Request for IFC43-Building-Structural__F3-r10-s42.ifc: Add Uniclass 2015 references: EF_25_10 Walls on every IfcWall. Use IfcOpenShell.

First a look at what the model holds.

```python
import ifcopenshell

model = ifcopenshell.open("IFC43-Building-Structural__F3-r10-s42.ifc")
print(model.schema)
print("classifications:", [c.Name for c in model.by_type("IfcClassification")])
for ifc_class in ("IfcDoor", "IfcRoof", "IfcStair", "IfcWall", "IfcWindow"):
    print(ifc_class, len(model.by_type(ifc_class)))
```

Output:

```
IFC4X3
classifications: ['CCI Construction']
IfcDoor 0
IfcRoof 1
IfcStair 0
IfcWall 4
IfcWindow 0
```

```python
import ifcopenshell
import ifcopenshell.api.classification

model = ifcopenshell.open("IFC43-Building-Structural__F3-r10-s42.ifc")

system = ifcopenshell.api.classification.add_classification(model, classification="Uniclass 2015")

codes = {
    "IfcWall": ("EF_25_10", "Walls"),
}
for ifc_class, (code, name) in codes.items():
    products = model.by_type(ifc_class)
    ifcopenshell.api.classification.add_reference(
        model, products=products, classification=system, identification=code, name=name
    )
    print(code, len(products))

model.write("IFC43-Building-Structural__F3-r10-s42_edited.ifc")
```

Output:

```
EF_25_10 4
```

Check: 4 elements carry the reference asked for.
